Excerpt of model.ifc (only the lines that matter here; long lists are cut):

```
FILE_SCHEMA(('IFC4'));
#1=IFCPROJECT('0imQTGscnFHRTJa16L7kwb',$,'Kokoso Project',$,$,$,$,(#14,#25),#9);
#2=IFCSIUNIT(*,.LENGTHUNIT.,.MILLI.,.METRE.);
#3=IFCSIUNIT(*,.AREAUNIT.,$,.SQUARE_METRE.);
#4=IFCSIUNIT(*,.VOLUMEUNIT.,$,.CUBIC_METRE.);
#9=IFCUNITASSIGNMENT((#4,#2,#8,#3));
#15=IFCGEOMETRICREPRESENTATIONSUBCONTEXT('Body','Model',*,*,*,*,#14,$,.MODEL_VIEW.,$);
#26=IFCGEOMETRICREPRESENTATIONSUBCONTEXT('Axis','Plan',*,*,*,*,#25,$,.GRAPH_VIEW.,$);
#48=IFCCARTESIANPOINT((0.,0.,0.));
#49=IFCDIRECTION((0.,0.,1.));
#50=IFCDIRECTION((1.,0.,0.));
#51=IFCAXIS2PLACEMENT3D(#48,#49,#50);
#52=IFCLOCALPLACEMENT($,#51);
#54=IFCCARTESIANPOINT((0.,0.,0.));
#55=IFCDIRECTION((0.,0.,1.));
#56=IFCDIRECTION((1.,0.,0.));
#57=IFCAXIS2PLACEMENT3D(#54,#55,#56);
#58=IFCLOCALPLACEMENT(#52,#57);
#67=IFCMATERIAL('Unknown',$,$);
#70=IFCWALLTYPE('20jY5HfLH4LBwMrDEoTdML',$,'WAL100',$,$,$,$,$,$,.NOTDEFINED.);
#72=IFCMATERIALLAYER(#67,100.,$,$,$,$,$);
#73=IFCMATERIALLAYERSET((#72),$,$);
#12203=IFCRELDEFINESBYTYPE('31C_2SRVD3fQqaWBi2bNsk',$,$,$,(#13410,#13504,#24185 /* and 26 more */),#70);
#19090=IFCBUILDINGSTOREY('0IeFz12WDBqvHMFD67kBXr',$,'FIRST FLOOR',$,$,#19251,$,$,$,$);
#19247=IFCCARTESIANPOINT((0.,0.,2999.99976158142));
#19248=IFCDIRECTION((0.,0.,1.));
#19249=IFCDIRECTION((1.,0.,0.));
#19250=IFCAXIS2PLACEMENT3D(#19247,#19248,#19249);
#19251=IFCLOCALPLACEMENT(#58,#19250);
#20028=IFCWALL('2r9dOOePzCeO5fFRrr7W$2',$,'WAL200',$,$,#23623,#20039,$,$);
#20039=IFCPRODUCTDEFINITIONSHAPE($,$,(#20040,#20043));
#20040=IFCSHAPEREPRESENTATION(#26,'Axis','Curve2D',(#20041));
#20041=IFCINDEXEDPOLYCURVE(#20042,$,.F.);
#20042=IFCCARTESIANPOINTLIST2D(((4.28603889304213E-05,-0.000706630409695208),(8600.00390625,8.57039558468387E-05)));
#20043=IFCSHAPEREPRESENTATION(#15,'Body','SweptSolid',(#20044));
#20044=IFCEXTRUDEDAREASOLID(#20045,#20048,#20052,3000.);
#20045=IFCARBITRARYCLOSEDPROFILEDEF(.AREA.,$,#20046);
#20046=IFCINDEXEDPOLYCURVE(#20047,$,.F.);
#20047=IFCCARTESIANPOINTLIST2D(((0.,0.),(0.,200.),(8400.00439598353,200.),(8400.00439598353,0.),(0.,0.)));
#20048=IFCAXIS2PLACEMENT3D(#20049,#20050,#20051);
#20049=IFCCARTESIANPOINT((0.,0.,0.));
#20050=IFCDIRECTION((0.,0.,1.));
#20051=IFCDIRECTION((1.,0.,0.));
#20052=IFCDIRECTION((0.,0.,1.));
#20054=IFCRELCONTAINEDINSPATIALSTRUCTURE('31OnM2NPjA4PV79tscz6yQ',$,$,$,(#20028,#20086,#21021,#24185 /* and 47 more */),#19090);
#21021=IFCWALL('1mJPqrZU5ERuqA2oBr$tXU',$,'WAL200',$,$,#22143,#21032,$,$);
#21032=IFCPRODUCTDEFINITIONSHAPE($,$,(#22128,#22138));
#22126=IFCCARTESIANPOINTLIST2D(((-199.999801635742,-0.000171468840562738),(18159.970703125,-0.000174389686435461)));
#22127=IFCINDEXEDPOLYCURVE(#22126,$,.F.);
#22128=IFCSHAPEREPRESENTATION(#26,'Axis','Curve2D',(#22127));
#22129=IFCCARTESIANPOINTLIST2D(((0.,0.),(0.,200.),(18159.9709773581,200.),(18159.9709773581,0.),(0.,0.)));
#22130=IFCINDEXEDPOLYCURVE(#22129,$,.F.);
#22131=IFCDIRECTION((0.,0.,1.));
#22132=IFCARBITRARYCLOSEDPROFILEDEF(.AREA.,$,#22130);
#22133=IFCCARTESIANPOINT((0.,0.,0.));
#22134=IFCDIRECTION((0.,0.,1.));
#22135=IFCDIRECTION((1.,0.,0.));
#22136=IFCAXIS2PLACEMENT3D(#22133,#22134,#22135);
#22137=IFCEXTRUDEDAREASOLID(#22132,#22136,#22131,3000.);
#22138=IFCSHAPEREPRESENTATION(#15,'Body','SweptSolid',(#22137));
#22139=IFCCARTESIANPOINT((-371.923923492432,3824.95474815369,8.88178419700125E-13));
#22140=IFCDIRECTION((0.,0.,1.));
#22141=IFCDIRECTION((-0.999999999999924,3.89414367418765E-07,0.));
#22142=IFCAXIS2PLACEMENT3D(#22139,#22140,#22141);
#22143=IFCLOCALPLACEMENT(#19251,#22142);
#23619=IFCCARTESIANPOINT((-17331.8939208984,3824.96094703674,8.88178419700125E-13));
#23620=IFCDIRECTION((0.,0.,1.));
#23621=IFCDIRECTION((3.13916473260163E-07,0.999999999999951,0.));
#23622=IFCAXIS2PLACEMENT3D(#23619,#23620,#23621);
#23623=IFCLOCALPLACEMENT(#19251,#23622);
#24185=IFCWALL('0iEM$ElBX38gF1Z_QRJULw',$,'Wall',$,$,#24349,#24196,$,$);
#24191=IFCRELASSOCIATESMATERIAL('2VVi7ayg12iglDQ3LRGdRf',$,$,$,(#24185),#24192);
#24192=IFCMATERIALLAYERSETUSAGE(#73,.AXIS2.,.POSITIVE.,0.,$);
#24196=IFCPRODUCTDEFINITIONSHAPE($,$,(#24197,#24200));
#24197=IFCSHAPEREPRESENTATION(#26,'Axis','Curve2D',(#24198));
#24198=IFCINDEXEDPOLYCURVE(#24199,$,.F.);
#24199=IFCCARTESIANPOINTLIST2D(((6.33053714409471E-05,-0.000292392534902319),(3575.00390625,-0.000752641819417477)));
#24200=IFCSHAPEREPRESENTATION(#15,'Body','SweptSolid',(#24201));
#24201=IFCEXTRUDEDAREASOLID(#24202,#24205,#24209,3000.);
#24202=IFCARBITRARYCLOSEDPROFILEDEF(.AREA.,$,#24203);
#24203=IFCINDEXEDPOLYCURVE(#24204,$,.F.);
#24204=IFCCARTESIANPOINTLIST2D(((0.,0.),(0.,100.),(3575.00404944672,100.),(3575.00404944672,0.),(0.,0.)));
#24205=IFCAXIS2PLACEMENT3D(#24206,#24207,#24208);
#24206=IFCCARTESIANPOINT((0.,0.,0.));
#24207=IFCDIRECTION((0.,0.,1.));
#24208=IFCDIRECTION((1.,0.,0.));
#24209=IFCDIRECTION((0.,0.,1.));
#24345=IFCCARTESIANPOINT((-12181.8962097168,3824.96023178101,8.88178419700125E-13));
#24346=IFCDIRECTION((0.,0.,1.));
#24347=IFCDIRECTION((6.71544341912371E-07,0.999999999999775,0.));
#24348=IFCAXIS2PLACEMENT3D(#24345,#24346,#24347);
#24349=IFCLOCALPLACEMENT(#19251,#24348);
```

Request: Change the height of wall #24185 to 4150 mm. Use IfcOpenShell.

```python
import ifcopenshell
import ifcopenshell.geom
import ifcopenshell.util.representation
import ifcopenshell.util.shape
import ifcopenshell.util.unit

model = ifcopenshell.open("model.ifc")
unit_scale = ifcopenshell.util.unit.calculate_unit_scale(model)
settings = ifcopenshell.geom.settings()


def volume(element):
    """Net volume in cubic metres, openings subtracted."""
    shape = ifcopenshell.geom.create_shape(settings, element)
    return ifcopenshell.util.shape.get_volume(shape.geometry)


wall = model.by_guid("0iEM$ElBX38gF1Z_QRJULw")
before = volume(wall)

body = ifcopenshell.util.representation.get_representation(wall, "Model", "Body")
solid = body.Items[0]
old_height = solid.Depth
solid.Depth = 4.15 / unit_scale
after = volume(wall)

print(f"height {old_height:g} -> {solid.Depth:g}, volume {before:.3f} -> {after:.3f} m3")

model.write("model_rev.ifc")
```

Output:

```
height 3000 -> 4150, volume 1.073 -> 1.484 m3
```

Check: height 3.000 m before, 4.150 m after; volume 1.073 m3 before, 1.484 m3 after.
